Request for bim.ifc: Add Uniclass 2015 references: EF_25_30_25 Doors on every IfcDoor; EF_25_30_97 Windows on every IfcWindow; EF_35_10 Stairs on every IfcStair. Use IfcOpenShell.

First a look at what the model holds.

```python
import ifcopenshell

model = ifcopenshell.open("bim.ifc")
print(model.schema)
print("classifications:", [c.Name for c in model.by_type("IfcClassification")])
for ifc_class in ("IfcDoor", "IfcRoof", "IfcStair", "IfcWall", "IfcWindow"):
    print(ifc_class, len(model.by_type(ifc_class)))
```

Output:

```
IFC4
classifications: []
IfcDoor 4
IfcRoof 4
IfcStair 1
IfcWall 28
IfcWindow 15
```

```python
import ifcopenshell
import ifcopenshell.api.classification

model = ifcopenshell.open("bim.ifc")

system = ifcopenshell.api.classification.add_classification(model, classification="Uniclass 2015")

codes = {
    "IfcDoor": ("EF_25_30_25", "Doors"),
    "IfcWindow": ("EF_25_30_97", "Windows"),
    "IfcStair": ("EF_35_10", "Stairs"),
}
for ifc_class, (code, name) in codes.items():
    products = model.by_type(ifc_class)
    ifcopenshell.api.classification.add_reference(
        model, products=products, classification=system, identification=code, name=name
    )
    print(code, len(products))

model.write("bim_edited.ifc")
```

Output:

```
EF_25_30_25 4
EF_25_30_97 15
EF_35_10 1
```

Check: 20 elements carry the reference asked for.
